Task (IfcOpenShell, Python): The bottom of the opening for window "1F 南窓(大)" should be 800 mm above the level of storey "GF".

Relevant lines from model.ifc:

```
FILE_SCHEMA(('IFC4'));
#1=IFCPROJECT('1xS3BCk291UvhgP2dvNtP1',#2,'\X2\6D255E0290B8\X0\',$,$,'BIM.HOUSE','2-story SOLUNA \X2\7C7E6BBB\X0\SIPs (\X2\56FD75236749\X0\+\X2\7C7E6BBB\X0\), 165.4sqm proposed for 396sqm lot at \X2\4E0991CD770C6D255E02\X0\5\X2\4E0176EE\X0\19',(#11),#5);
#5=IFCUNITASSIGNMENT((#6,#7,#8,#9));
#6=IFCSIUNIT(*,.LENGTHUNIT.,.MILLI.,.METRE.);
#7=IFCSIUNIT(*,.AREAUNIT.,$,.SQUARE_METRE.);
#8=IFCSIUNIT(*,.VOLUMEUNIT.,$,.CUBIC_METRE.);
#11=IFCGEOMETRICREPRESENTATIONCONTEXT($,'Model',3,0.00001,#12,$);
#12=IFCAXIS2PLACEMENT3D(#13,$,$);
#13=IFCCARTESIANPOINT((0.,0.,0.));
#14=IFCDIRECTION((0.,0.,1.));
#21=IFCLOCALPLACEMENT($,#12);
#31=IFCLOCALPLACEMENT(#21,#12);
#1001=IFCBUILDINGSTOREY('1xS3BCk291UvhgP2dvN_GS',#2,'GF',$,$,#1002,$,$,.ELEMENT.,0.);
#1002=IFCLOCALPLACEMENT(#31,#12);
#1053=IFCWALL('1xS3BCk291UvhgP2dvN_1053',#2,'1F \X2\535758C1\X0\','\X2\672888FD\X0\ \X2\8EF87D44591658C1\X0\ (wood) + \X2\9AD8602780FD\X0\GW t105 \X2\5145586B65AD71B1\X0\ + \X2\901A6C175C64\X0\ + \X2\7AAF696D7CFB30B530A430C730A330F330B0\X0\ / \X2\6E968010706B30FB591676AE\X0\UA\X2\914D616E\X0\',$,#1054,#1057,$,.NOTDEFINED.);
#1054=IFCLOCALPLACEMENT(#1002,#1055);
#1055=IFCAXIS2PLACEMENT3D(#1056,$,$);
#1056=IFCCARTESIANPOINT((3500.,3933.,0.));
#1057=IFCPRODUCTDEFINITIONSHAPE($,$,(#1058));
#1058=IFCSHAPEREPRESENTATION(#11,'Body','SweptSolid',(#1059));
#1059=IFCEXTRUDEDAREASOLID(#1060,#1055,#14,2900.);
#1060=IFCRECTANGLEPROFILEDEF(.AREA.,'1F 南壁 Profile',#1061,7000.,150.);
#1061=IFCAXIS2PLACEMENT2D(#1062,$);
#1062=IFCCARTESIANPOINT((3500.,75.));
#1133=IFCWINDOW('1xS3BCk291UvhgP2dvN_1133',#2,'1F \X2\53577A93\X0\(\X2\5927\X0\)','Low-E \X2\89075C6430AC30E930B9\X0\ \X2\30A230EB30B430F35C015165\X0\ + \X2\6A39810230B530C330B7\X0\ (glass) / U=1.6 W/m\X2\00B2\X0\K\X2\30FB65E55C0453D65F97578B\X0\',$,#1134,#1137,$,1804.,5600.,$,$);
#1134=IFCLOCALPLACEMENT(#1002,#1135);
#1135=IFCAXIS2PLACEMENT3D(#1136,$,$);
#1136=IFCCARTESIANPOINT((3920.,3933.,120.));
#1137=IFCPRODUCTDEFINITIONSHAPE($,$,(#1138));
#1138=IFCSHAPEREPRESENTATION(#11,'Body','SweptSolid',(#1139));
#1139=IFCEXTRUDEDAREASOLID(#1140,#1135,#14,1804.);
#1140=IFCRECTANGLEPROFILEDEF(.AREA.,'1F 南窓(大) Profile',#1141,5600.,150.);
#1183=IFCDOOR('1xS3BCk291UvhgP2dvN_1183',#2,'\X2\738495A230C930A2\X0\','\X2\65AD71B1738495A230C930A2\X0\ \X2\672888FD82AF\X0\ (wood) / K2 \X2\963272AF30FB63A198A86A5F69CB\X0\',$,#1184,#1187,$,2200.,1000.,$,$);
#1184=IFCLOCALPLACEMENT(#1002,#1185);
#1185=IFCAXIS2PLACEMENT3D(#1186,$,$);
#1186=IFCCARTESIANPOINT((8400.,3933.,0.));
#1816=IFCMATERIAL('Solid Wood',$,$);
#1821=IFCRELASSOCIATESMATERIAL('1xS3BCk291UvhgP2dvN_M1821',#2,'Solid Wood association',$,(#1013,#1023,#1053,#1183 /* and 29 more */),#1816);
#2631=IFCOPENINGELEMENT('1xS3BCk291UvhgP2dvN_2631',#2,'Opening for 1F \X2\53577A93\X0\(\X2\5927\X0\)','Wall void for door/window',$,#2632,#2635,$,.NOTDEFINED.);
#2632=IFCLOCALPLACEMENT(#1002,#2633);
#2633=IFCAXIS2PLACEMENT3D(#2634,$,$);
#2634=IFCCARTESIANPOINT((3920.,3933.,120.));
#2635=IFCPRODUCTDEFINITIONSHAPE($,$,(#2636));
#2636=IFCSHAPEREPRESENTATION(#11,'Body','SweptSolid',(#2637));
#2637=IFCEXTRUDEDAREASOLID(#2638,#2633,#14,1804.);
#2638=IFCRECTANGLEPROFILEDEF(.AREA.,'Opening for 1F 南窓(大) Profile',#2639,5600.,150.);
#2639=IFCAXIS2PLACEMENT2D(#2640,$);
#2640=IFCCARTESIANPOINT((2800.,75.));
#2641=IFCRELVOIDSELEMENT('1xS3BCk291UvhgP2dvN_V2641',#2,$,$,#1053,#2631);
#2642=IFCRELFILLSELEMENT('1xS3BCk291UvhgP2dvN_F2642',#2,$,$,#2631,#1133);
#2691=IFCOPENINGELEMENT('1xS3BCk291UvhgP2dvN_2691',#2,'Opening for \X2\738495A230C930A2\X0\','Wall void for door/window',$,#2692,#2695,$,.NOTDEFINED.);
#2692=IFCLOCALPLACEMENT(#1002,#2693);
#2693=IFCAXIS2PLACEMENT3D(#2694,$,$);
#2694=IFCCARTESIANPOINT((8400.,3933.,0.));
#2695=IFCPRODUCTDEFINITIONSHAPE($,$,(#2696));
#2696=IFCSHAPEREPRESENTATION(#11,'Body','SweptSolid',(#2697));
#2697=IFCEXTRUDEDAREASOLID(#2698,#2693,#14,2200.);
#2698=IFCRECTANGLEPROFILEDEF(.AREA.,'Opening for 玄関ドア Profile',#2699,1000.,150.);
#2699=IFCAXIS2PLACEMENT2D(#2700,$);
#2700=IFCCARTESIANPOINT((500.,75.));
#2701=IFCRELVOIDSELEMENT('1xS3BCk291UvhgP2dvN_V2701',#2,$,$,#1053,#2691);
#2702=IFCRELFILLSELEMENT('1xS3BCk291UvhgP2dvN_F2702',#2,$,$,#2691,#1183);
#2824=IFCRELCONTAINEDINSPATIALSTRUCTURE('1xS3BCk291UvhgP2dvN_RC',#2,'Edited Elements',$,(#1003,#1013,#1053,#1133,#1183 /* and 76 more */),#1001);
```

```python
import numpy as np
import ifcopenshell
import ifcopenshell.api.geometry
import ifcopenshell.geom
import ifcopenshell.util.element
import ifcopenshell.util.placement
import ifcopenshell.util.shape
import ifcopenshell.util.unit

model = ifcopenshell.open("model.ifc")
unit_scale = ifcopenshell.util.unit.calculate_unit_scale(model)

window = model.by_id(1133)
opening = window.FillsVoids[0].RelatingOpeningElement
storey = ifcopenshell.util.element.get_container(window, ifc_class="IfcBuildingStorey")
level = ifcopenshell.util.placement.get_local_placement(storey.ObjectPlacement)[2, 3]

# The opening's origin need not be at the sill, so measure its lowest point.
shape = ifcopenshell.geom.create_shape(ifcopenshell.geom.settings(), opening)
bottom = ifcopenshell.util.shape.get_shape_bottom_elevation(shape, shape.geometry) / unit_scale
dz = level + 800.0 - bottom

shift = np.array([0.0, 0.0, dz])
# The window is not placed relative to its opening, so move both.
for product in (opening, window):
    matrix = ifcopenshell.util.placement.get_local_placement(product.ObjectPlacement)
    matrix[:3, 3] += shift
    ifcopenshell.api.geometry.edit_object_placement(model, product=product, matrix=matrix, is_si=False)

print(f"moved by {dz * unit_scale:+.3f} m")

model.write("model_v2.ifc")
```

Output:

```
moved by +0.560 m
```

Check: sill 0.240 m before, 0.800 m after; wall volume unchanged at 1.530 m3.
